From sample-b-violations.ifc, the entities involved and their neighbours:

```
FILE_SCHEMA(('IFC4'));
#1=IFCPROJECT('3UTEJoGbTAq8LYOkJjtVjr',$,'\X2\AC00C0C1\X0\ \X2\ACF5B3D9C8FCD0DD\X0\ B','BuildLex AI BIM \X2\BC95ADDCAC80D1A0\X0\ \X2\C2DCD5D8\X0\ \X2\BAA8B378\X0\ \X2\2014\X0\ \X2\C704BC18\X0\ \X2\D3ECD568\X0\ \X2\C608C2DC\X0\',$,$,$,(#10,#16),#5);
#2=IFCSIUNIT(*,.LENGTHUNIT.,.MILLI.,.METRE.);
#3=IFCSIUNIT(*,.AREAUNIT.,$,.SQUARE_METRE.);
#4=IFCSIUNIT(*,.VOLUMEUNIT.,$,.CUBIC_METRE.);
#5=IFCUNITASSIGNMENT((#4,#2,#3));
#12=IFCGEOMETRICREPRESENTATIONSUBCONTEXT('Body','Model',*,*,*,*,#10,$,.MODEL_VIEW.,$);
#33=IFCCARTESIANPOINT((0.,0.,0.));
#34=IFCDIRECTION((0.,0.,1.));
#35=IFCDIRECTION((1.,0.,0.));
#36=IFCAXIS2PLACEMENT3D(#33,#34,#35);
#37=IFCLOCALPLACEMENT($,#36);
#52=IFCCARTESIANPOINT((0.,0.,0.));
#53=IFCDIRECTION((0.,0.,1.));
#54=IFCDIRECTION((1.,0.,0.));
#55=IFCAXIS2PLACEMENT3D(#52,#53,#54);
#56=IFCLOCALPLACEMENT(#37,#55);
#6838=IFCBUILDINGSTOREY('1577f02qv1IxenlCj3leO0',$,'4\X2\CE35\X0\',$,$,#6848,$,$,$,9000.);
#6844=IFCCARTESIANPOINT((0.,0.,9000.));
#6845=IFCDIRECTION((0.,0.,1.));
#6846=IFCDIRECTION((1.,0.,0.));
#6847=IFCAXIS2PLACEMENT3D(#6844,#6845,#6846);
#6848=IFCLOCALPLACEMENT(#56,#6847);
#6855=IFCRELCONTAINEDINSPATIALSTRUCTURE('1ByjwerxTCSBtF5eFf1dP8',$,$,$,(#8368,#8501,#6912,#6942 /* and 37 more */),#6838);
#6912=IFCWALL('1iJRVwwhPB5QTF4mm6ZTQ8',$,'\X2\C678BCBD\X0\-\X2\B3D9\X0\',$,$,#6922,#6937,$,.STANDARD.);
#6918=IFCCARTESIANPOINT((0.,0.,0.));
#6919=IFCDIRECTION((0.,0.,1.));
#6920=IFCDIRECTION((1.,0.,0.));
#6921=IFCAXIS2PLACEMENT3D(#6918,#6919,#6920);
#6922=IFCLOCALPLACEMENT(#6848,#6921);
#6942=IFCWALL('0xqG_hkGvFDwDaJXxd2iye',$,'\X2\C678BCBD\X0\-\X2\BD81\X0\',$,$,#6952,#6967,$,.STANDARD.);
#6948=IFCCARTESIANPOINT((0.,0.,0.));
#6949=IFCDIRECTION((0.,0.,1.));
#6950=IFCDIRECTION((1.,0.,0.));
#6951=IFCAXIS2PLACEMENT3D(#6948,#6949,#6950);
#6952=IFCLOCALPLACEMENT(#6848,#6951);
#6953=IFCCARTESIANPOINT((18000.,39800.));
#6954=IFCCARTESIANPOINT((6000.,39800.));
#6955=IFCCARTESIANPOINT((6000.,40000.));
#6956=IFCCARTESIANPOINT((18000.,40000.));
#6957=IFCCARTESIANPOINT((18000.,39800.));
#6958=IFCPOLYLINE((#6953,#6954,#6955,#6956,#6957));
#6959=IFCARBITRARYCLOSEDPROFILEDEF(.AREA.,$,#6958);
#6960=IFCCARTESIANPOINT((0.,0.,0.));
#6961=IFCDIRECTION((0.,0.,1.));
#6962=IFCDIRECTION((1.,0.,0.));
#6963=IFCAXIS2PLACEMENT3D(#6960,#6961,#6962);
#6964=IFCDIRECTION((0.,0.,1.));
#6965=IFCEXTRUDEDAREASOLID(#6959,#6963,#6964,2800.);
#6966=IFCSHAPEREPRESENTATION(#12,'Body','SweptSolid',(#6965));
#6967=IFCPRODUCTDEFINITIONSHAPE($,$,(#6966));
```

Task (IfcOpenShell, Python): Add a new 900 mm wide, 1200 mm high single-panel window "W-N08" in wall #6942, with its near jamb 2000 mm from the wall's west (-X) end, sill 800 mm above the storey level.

```python
import numpy as np
import ifcopenshell
import ifcopenshell.api.feature
import ifcopenshell.api.geometry
import ifcopenshell.api.root
import ifcopenshell.api.spatial
import ifcopenshell.geom
import ifcopenshell.util.element
import ifcopenshell.util.placement
import ifcopenshell.util.representation
import ifcopenshell.util.shape
import ifcopenshell.util.unit

model = ifcopenshell.open("sample-b-violations.ifc")
unit_scale = ifcopenshell.util.unit.calculate_unit_scale(model)
settings = ifcopenshell.geom.settings()


def volume(element):
    """Net volume in cubic metres, openings subtracted."""
    shape = ifcopenshell.geom.create_shape(settings, element)
    return ifcopenshell.util.shape.get_volume(shape.geometry)


wall = model.by_guid("0xqG_hkGvFDwDaJXxd2iye")
storey = ifcopenshell.util.element.get_container(wall, ifc_class="IfcBuildingStorey")
context = ifcopenshell.util.representation.get_context(model, "Model", "Body", "MODEL_VIEW")
before = volume(wall)

width, height, from_end, sill = 0.9, 1.2, 2, 0.8  # metres

# The wall runs along its own X axis, and the end named is its -X end.
wall_shape = ifcopenshell.geom.create_shape(settings, wall)
x, y, z = ifcopenshell.util.shape.get_vertices(wall_shape.geometry).T
start = x.min() + from_end
face, thickness = float(y.min()), float(y.max() - y.min())
wall_matrix = ifcopenshell.util.placement.get_local_placement(wall.ObjectPlacement)
level = ifcopenshell.util.placement.get_local_placement(storey.ObjectPlacement)[2, 3]


def in_wall(x, y):
    """Placement at x, y metres in the wall's axes, at sill height."""
    matrix = wall_matrix.copy()
    matrix[:, 3] = wall_matrix @ np.array([x / unit_scale, y / unit_scale, 0.0, 1.0])
    matrix[2, 3] = level + sill / unit_scale
    return matrix


# Opening: a box that overshoots both wall faces by 50 mm.
opening = ifcopenshell.api.root.create_entity(model, ifc_class="IfcOpeningElement", predefined_type="OPENING")
box = ifcopenshell.api.geometry.add_wall_representation(
    model, context=context, length=width, height=height, thickness=thickness + 0.1
)
ifcopenshell.api.geometry.assign_representation(model, product=opening, representation=box)
ifcopenshell.api.geometry.edit_object_placement(model, product=opening, matrix=in_wall(start, face - 0.05), is_si=False)
ifcopenshell.api.feature.add_feature(model, feature=opening, element=wall)

window = ifcopenshell.api.root.create_entity(model, ifc_class="IfcWindow", name="W-N08", predefined_type="WINDOW")
window.OverallWidth, window.OverallHeight = width / unit_scale, height / unit_scale
window.PartitioningType = "SINGLE_PANEL"
body = ifcopenshell.api.geometry.add_window_representation(
    model,
    context=context,
    overall_width=window.OverallWidth,
    overall_height=window.OverallHeight,
    partition_type="SINGLE_PANEL",
)
ifcopenshell.api.geometry.assign_representation(model, product=window, representation=body)
ifcopenshell.api.spatial.assign_container(model, products=[window], relating_structure=storey)
ifcopenshell.api.feature.add_filling(model, opening=opening, element=window)

# Centre the window in the wall's thickness.
ifcopenshell.api.geometry.edit_object_placement(model, product=window, matrix=in_wall(start, face), is_si=False)
window_shape = ifcopenshell.geom.create_shape(settings, window)
depth = ifcopenshell.util.shape.get_vertices(window_shape.geometry)[:, 1]
offset = face + thickness / 2 - (depth.min() + depth.max()) / 2
ifcopenshell.api.geometry.edit_object_placement(model, product=window, matrix=in_wall(start, offset), is_si=False)

after = volume(wall)

print(f"wall volume {before:.3f} -> {after:.3f} m3")

model.write("sample-b-violations-out.ifc")
```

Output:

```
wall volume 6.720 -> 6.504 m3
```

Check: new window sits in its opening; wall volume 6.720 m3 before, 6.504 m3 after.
